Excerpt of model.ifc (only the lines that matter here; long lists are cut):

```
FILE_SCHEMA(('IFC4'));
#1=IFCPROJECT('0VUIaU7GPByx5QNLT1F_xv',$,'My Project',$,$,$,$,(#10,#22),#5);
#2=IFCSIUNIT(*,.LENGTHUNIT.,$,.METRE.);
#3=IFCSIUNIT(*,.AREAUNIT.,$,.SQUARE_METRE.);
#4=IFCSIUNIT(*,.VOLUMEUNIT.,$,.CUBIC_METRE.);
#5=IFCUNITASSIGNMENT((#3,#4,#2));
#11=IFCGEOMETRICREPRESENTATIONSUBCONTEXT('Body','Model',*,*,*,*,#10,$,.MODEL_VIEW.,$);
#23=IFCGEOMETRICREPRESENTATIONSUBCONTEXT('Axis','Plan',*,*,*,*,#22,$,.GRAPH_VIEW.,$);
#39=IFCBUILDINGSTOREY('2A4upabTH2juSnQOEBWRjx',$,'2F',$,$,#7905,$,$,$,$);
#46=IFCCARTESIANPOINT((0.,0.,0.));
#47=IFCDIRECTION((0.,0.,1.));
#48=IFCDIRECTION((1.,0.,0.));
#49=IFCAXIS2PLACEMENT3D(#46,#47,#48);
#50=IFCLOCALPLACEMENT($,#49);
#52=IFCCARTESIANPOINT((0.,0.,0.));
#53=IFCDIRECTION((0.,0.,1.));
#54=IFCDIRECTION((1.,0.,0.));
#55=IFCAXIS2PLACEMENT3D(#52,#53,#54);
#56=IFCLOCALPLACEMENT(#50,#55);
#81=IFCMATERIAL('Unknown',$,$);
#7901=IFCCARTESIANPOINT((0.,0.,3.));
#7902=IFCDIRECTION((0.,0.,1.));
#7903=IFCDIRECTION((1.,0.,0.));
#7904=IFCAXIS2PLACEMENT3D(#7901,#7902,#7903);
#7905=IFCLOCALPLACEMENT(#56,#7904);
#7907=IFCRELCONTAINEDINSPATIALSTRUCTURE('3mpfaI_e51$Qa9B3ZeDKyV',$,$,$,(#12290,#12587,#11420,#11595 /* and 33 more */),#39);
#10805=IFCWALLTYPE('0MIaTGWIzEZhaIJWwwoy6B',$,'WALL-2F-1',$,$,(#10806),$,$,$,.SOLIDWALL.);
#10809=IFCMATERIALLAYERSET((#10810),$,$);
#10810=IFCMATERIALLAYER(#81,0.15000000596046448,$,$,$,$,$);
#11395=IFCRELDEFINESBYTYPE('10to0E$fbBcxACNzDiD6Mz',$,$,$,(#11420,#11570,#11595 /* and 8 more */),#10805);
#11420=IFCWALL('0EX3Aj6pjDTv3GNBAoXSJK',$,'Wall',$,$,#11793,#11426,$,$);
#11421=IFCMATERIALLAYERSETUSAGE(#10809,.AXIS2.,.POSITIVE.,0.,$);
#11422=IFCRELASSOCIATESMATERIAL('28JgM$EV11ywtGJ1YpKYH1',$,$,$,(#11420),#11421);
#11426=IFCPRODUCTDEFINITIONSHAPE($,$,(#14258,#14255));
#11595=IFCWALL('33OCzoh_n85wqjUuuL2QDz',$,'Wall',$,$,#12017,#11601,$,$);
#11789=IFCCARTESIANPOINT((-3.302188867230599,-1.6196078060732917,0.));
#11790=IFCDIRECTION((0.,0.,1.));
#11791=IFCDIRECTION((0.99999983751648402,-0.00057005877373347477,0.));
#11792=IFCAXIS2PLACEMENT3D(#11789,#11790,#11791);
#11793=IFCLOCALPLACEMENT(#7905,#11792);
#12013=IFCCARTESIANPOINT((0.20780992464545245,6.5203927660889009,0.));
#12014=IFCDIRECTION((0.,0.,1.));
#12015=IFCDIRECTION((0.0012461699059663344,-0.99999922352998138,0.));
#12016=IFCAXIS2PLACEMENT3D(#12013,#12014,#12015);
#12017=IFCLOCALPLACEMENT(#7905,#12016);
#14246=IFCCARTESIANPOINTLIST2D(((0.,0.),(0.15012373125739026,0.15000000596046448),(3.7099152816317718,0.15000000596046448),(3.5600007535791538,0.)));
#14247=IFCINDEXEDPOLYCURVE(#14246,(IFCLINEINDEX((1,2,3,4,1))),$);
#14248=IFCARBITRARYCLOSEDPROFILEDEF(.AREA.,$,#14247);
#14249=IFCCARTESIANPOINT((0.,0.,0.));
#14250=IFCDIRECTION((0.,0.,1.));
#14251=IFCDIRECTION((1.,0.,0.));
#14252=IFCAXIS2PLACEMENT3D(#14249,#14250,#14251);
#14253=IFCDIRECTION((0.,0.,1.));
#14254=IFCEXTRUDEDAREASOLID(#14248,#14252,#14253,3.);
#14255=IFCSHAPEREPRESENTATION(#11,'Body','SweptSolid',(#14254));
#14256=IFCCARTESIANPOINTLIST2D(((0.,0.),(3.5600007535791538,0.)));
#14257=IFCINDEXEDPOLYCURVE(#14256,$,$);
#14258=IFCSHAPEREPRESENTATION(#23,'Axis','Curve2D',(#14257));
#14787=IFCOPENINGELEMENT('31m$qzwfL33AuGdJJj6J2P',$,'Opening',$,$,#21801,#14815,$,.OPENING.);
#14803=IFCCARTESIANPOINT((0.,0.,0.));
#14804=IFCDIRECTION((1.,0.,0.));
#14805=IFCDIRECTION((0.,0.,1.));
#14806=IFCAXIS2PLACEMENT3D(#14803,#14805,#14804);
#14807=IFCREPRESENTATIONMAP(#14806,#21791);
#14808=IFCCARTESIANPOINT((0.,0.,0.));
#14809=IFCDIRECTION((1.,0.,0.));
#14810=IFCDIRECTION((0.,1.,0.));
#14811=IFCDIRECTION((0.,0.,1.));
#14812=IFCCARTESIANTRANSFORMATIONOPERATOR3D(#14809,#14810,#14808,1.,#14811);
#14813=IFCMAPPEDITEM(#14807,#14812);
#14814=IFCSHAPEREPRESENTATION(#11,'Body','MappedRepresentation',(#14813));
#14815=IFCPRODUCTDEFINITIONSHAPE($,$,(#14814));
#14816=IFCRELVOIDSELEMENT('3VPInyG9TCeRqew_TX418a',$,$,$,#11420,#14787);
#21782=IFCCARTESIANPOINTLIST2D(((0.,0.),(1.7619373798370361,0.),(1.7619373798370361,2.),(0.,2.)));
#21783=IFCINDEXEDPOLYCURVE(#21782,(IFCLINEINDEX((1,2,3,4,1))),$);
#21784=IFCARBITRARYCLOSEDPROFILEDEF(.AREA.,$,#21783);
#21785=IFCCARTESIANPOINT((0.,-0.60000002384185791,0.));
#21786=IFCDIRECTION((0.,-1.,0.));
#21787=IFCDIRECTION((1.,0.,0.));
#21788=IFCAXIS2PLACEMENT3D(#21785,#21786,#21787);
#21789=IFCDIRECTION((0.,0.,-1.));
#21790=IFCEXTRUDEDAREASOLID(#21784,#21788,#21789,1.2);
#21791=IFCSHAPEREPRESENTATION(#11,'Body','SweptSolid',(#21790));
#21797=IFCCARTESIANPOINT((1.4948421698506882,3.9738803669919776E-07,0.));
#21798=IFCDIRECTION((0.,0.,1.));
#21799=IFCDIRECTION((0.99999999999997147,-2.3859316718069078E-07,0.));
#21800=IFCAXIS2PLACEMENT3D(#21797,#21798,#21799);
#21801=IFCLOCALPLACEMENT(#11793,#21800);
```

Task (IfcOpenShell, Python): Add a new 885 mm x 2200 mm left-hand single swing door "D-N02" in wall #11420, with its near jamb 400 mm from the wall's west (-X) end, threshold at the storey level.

```python
import numpy as np
import ifcopenshell
import ifcopenshell.api.feature
import ifcopenshell.api.geometry
import ifcopenshell.api.root
import ifcopenshell.api.spatial
import ifcopenshell.geom
import ifcopenshell.util.element
import ifcopenshell.util.placement
import ifcopenshell.util.representation
import ifcopenshell.util.shape
import ifcopenshell.util.unit

model = ifcopenshell.open("model.ifc")
unit_scale = ifcopenshell.util.unit.calculate_unit_scale(model)
settings = ifcopenshell.geom.settings()


def volume(element):
    """Net volume in cubic metres, openings subtracted."""
    shape = ifcopenshell.geom.create_shape(settings, element)
    return ifcopenshell.util.shape.get_volume(shape.geometry)


wall = model.by_guid("0EX3Aj6pjDTv3GNBAoXSJK")
storey = ifcopenshell.util.element.get_container(wall, ifc_class="IfcBuildingStorey")
context = ifcopenshell.util.representation.get_context(model, "Model", "Body", "MODEL_VIEW")
before = volume(wall)

width, height, from_end, sill = 0.885, 2.2, 0.4, 0.0  # metres

# The wall runs along its own X axis, and the end named is its -X end.
wall_shape = ifcopenshell.geom.create_shape(settings, wall)
x, y, z = ifcopenshell.util.shape.get_vertices(wall_shape.geometry).T
start = x.min() + from_end
face, thickness = float(y.min()), float(y.max() - y.min())
wall_matrix = ifcopenshell.util.placement.get_local_placement(wall.ObjectPlacement)
level = ifcopenshell.util.placement.get_local_placement(storey.ObjectPlacement)[2, 3]


def in_wall(x, y):
    """Placement at x, y metres in the wall's axes, at sill height."""
    matrix = wall_matrix.copy()
    matrix[:, 3] = wall_matrix @ np.array([x / unit_scale, y / unit_scale, 0.0, 1.0])
    matrix[2, 3] = level + sill / unit_scale
    return matrix


# Opening: a box that overshoots both wall faces by 50 mm.
opening = ifcopenshell.api.root.create_entity(model, ifc_class="IfcOpeningElement", predefined_type="OPENING")
box = ifcopenshell.api.geometry.add_wall_representation(
    model, context=context, length=width, height=height, thickness=thickness + 0.1
)
ifcopenshell.api.geometry.assign_representation(model, product=opening, representation=box)
ifcopenshell.api.geometry.edit_object_placement(model, product=opening, matrix=in_wall(start, face - 0.05), is_si=False)
ifcopenshell.api.feature.add_feature(model, feature=opening, element=wall)

door = ifcopenshell.api.root.create_entity(model, ifc_class="IfcDoor", name="D-N02", predefined_type="DOOR")
door.OverallWidth, door.OverallHeight = width / unit_scale, height / unit_scale
door.OperationType = "SINGLE_SWING_LEFT"
body = ifcopenshell.api.geometry.add_door_representation(
    model,
    context=context,
    overall_width=door.OverallWidth,
    overall_height=door.OverallHeight,
    operation_type="SINGLE_SWING_LEFT",
    lining_properties={"LiningDepth": thickness / unit_scale, "ThresholdDepth": thickness / unit_scale},
)
ifcopenshell.api.geometry.assign_representation(model, product=door, representation=body)
ifcopenshell.api.spatial.assign_container(model, products=[door], relating_structure=storey)
ifcopenshell.api.feature.add_filling(model, opening=opening, element=door)

# The lining spans the wall, so the door starts at the wall face.
ifcopenshell.api.geometry.edit_object_placement(model, product=door, matrix=in_wall(start, face), is_si=False)

after = volume(wall)

print(f"wall volume {before:.3f} -> {after:.3f} m3")

model.write("model_updated.ifc")
```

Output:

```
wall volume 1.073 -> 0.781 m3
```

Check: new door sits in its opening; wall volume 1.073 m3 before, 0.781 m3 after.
